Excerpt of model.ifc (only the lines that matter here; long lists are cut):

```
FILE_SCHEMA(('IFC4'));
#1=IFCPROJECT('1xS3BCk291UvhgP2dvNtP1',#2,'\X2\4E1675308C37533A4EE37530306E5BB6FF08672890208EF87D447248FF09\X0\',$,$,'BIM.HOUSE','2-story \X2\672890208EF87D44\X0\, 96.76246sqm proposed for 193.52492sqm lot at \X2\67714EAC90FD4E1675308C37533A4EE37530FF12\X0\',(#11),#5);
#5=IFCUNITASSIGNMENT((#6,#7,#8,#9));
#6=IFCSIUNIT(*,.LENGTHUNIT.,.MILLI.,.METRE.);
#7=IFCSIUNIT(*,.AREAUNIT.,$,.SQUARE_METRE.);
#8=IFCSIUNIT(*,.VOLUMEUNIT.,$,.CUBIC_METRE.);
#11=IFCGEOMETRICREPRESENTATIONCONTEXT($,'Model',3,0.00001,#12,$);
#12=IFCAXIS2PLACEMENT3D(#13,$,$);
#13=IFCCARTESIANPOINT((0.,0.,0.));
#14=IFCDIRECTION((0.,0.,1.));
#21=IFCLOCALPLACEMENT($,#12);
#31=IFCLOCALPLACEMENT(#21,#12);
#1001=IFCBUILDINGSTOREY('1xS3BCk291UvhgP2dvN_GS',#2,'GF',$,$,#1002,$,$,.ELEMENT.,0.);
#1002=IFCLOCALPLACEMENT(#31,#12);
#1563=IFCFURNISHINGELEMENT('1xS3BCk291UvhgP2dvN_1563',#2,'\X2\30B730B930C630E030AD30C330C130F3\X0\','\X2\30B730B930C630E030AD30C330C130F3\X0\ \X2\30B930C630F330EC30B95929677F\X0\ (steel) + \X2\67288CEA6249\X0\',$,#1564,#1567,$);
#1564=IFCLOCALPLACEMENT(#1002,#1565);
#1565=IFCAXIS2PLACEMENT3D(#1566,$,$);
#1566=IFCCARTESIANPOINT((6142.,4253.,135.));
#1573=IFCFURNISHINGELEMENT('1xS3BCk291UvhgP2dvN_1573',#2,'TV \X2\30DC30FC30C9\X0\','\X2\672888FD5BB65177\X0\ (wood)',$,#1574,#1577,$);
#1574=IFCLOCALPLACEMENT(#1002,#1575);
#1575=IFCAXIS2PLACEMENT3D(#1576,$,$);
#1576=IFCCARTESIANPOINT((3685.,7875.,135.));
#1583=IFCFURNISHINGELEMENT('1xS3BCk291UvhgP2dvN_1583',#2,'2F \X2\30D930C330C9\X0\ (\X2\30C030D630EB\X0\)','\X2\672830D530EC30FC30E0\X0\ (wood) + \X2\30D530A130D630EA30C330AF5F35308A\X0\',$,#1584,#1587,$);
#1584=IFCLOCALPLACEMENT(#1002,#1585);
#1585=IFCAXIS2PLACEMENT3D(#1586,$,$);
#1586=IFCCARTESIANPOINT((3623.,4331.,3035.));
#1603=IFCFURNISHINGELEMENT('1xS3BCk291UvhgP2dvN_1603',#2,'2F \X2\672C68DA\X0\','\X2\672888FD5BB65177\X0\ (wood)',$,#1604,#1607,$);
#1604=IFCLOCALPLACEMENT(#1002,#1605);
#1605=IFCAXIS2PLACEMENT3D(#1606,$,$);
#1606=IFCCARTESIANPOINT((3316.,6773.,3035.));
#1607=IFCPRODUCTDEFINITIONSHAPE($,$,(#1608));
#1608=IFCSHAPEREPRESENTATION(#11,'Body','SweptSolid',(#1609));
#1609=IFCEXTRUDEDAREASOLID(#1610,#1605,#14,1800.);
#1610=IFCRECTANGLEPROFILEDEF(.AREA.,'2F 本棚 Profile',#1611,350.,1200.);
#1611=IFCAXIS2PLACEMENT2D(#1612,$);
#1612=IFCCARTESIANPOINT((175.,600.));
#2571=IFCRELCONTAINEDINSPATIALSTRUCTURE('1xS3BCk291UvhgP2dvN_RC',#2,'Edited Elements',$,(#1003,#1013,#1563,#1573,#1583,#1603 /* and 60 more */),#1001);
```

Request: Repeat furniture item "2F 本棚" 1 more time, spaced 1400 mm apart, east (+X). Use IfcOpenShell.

```python
import numpy as np
import ifcopenshell
import ifcopenshell.api.geometry
import ifcopenshell.api.root
import ifcopenshell.util.element
import ifcopenshell.util.placement
import ifcopenshell.util.unit

model = ifcopenshell.open("model.ifc")
unit_scale = ifcopenshell.util.unit.calculate_unit_scale(model)


def reuse_history(source, copy):
    """copy_class also copies each property set's owner history, people and application; keep the originals."""
    for rel in copy.IsDefinedBy:
        if rel.is_a("IfcRelDefinesByProperties") and (history := rel.RelatingPropertyDefinition.OwnerHistory):
            rel.RelatingPropertyDefinition.OwnerHistory = source.OwnerHistory
            ifcopenshell.util.element.remove_deep2(model, history)


source = model.by_guid("1xS3BCk291UvhgP2dvN_1603")
base = ifcopenshell.util.placement.get_local_placement(source.ObjectPlacement)
step = np.array([1.0, 0.0, 0.0]) * 1.4 / unit_scale

for i in range(1, 2):
    copy = ifcopenshell.api.root.copy_class(model, product=source)
    copy.Representation = ifcopenshell.util.element.copy_deep(
        model, source.Representation, exclude=["IfcGeometricRepresentationContext", "IfcRepresentationMap"]
    )
    reuse_history(source, copy)
    matrix = base.copy()
    matrix[:3, 3] += i * step
    print("added at", matrix[:3, 3].round(3) + 0.0)
    ifcopenshell.api.geometry.edit_object_placement(model, product=copy, matrix=matrix, is_si=False)

model.write("model_v2.ifc")
```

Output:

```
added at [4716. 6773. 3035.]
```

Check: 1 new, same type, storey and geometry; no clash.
